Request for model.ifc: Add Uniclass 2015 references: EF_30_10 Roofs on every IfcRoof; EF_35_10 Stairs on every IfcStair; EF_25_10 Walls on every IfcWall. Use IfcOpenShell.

First a look at what the model holds.

```python
import ifcopenshell

model = ifcopenshell.open("model.ifc")
print(model.schema)
print("classifications:", [c.Name for c in model.by_type("IfcClassification")])
for ifc_class in ("IfcDoor", "IfcRoof", "IfcStair", "IfcWall", "IfcWindow"):
    print(ifc_class, len(model.by_type(ifc_class)))
```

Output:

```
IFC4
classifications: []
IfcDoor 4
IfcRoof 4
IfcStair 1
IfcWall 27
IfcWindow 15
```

```python
import ifcopenshell
import ifcopenshell.api.classification

model = ifcopenshell.open("model.ifc")

system = ifcopenshell.api.classification.add_classification(model, classification="Uniclass 2015")

codes = {
    "IfcRoof": ("EF_30_10", "Roofs"),
    "IfcStair": ("EF_35_10", "Stairs"),
    "IfcWall": ("EF_25_10", "Walls"),
}
for ifc_class, (code, name) in codes.items():
    products = model.by_type(ifc_class)
    ifcopenshell.api.classification.add_reference(
        model, products=products, classification=system, identification=code, name=name
    )
    print(code, len(products))

model.write("model-out.ifc")
```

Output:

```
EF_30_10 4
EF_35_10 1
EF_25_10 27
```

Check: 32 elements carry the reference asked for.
